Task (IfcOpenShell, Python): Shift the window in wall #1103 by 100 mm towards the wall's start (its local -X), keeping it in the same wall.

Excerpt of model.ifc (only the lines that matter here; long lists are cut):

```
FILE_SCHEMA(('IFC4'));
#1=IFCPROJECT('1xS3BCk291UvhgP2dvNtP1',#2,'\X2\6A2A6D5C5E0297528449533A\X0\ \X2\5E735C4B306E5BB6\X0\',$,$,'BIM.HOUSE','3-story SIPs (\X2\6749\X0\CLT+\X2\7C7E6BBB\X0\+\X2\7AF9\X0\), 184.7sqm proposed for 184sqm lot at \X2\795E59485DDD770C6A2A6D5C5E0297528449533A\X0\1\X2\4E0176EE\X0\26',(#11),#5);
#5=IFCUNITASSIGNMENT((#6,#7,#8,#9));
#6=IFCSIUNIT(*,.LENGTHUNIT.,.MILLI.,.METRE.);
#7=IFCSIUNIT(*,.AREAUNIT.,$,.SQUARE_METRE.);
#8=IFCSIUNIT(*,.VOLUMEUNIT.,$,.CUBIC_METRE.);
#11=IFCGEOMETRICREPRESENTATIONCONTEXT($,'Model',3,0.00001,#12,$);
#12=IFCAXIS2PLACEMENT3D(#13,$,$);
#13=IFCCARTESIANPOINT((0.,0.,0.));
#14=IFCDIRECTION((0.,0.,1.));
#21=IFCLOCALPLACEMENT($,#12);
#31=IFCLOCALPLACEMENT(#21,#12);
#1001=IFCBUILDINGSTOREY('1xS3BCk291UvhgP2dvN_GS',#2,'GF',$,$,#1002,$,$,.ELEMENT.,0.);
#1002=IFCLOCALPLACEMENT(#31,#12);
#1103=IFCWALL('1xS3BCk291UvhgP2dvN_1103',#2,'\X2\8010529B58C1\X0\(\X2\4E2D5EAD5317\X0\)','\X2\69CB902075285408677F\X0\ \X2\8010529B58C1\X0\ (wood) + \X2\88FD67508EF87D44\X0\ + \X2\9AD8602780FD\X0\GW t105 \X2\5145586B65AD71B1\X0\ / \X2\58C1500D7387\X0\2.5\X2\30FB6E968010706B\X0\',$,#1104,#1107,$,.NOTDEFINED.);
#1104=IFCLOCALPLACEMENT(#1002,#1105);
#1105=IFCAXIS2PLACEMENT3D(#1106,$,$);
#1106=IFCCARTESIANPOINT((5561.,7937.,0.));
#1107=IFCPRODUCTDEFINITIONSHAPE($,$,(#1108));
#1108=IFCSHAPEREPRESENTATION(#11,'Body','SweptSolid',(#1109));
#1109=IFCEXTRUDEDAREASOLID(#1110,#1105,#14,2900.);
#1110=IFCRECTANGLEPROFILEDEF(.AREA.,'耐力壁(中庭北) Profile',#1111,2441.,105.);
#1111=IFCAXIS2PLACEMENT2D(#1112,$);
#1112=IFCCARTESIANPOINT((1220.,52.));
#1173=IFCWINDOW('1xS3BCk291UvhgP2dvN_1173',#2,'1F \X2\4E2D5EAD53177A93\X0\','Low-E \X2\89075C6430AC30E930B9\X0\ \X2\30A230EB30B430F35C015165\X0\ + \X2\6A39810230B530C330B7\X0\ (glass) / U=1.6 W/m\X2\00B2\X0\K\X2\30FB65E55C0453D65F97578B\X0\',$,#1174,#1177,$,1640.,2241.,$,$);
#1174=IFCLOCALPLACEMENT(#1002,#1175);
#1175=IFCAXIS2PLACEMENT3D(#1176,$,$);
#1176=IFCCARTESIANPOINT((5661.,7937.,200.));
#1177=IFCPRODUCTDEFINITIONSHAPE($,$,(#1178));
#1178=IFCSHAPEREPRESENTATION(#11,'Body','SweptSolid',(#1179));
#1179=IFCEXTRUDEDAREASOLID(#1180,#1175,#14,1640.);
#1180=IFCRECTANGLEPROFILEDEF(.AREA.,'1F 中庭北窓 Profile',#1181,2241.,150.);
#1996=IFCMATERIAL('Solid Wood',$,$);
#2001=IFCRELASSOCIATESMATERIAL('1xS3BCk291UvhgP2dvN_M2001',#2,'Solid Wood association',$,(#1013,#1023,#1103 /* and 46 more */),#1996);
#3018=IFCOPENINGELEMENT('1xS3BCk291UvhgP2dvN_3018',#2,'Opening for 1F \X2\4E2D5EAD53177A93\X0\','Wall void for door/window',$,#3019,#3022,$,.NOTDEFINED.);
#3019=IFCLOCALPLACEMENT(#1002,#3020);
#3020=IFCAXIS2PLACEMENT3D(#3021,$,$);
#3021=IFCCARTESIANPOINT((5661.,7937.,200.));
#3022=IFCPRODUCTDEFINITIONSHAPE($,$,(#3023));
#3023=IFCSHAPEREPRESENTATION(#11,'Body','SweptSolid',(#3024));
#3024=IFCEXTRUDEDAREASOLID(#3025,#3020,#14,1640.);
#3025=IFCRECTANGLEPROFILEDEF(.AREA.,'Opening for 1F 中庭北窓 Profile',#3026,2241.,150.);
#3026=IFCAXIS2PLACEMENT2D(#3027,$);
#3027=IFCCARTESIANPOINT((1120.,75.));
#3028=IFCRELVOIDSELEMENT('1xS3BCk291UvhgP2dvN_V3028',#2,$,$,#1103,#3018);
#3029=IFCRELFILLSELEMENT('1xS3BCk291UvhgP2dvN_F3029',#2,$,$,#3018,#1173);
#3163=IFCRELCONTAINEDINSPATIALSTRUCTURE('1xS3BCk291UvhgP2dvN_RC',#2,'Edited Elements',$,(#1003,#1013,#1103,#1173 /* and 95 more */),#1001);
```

```python
import ifcopenshell
import ifcopenshell.api.geometry
import ifcopenshell.util.placement

model = ifcopenshell.open("model.ifc")

window = model.by_guid("1xS3BCk291UvhgP2dvN_1173")
opening = window.FillsVoids[0].RelatingOpeningElement
wall = opening.VoidsElements[0].RelatingBuildingElement

wall_matrix = ifcopenshell.util.placement.get_local_placement(wall.ObjectPlacement)
shift = wall_matrix[:3, 0] * -100.0
before = ifcopenshell.util.placement.get_local_placement(window.ObjectPlacement)[:3, 3].copy()

# The window is not placed relative to its opening, so move both.
for product in (opening, window):
    matrix = ifcopenshell.util.placement.get_local_placement(product.ObjectPlacement)
    matrix[:3, 3] += shift
    ifcopenshell.api.geometry.edit_object_placement(model, product=product, matrix=matrix, is_si=False)

after = ifcopenshell.util.placement.get_local_placement(window.ObjectPlacement)[:3, 3]
print("window moved by", (after - before).round(3) + 0.0)

model.write("model_edited.ifc")
```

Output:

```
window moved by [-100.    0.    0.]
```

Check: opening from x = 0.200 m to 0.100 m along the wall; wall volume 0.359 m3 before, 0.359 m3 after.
